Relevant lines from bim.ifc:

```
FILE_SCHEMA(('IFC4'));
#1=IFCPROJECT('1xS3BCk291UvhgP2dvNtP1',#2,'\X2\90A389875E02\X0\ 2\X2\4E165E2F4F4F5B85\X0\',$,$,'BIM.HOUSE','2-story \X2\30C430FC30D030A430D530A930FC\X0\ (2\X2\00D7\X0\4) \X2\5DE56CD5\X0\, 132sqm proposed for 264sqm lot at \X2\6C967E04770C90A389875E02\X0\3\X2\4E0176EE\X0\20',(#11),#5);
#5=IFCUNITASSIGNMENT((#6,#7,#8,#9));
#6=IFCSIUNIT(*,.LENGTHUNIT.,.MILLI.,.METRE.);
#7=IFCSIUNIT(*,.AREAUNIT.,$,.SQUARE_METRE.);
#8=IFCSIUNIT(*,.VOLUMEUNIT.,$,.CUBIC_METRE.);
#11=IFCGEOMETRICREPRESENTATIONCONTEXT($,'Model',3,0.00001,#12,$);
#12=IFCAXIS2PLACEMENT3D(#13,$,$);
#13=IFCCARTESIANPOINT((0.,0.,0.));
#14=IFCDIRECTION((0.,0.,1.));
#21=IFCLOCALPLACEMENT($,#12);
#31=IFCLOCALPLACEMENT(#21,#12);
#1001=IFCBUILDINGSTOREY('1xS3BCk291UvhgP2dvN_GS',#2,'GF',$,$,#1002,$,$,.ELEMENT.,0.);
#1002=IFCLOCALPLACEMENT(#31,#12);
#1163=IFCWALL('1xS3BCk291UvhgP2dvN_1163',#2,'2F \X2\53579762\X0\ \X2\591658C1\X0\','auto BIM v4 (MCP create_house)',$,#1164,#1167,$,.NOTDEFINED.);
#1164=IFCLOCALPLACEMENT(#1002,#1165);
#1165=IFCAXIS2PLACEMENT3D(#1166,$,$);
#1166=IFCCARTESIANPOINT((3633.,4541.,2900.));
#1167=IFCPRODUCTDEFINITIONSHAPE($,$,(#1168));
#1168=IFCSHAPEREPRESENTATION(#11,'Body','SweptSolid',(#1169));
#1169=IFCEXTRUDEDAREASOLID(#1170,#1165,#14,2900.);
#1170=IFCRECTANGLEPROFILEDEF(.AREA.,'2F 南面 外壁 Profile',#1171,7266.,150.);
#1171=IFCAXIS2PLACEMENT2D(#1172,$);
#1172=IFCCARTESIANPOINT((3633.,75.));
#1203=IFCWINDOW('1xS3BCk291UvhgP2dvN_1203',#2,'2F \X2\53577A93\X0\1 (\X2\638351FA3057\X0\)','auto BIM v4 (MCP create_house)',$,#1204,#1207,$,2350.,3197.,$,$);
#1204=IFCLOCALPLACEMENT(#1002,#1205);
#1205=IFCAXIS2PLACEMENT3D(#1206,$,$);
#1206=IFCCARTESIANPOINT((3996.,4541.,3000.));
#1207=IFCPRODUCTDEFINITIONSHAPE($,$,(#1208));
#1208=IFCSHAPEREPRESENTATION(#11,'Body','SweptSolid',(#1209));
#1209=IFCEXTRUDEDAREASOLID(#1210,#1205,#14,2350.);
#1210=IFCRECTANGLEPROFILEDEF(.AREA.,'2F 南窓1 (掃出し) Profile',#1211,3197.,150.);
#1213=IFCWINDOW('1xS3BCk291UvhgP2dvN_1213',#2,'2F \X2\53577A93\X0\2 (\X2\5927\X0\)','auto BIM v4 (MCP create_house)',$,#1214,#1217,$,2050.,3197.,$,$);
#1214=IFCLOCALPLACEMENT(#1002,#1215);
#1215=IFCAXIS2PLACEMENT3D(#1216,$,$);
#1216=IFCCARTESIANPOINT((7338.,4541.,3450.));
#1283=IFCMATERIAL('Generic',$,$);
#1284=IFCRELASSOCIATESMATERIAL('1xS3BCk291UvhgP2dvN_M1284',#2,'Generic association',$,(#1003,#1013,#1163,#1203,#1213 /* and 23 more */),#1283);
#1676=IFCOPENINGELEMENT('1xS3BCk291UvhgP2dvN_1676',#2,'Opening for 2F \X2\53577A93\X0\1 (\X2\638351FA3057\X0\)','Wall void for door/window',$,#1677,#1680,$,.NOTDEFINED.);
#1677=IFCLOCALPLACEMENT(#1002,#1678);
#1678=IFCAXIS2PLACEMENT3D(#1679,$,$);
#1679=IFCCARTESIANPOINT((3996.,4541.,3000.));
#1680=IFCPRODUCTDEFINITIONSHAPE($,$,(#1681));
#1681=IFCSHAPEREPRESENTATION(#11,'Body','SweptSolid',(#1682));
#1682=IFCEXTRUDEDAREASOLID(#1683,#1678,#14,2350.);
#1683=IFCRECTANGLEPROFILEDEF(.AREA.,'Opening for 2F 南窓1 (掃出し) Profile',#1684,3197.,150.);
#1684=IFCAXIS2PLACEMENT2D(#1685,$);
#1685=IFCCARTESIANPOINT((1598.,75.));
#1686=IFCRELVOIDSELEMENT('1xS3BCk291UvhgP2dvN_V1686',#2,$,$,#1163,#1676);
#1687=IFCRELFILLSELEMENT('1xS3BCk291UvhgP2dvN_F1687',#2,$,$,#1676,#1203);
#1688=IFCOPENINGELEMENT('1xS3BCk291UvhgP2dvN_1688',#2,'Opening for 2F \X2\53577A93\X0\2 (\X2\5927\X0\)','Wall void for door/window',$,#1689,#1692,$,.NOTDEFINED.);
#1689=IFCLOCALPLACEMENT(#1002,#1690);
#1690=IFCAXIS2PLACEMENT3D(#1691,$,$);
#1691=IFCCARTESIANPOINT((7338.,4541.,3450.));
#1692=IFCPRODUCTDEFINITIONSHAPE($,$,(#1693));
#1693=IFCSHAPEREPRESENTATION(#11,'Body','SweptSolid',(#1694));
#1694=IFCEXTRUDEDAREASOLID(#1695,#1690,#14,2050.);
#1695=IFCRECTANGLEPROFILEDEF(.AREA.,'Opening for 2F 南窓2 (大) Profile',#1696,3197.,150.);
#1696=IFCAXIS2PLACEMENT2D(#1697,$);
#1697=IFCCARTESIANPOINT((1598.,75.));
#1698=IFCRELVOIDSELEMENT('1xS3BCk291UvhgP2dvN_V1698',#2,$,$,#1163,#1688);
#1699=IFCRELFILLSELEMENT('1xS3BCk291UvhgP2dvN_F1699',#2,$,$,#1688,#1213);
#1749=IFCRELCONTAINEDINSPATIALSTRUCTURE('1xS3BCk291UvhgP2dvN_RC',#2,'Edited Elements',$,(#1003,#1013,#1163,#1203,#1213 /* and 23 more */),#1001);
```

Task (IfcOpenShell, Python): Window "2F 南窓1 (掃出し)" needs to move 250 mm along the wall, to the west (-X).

```python
import ifcopenshell
import ifcopenshell.api.geometry
import ifcopenshell.util.placement

model = ifcopenshell.open("bim.ifc")

window = model.by_id(1203)
opening = window.FillsVoids[0].RelatingOpeningElement
wall = opening.VoidsElements[0].RelatingBuildingElement

wall_matrix = ifcopenshell.util.placement.get_local_placement(wall.ObjectPlacement)
shift = wall_matrix[:3, 0] * -250.0
before = ifcopenshell.util.placement.get_local_placement(window.ObjectPlacement)[:3, 3].copy()

# The window is not placed relative to its opening, so move both.
for product in (opening, window):
    matrix = ifcopenshell.util.placement.get_local_placement(product.ObjectPlacement)
    matrix[:3, 3] += shift
    ifcopenshell.api.geometry.edit_object_placement(model, product=product, matrix=matrix, is_si=False)

after = ifcopenshell.util.placement.get_local_placement(window.ObjectPlacement)[:3, 3]
print("window moved by", (after - before).round(3) + 0.0)

model.write("bim_rev.ifc")
```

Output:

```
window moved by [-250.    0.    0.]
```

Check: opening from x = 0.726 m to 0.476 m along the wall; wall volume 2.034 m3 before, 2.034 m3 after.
